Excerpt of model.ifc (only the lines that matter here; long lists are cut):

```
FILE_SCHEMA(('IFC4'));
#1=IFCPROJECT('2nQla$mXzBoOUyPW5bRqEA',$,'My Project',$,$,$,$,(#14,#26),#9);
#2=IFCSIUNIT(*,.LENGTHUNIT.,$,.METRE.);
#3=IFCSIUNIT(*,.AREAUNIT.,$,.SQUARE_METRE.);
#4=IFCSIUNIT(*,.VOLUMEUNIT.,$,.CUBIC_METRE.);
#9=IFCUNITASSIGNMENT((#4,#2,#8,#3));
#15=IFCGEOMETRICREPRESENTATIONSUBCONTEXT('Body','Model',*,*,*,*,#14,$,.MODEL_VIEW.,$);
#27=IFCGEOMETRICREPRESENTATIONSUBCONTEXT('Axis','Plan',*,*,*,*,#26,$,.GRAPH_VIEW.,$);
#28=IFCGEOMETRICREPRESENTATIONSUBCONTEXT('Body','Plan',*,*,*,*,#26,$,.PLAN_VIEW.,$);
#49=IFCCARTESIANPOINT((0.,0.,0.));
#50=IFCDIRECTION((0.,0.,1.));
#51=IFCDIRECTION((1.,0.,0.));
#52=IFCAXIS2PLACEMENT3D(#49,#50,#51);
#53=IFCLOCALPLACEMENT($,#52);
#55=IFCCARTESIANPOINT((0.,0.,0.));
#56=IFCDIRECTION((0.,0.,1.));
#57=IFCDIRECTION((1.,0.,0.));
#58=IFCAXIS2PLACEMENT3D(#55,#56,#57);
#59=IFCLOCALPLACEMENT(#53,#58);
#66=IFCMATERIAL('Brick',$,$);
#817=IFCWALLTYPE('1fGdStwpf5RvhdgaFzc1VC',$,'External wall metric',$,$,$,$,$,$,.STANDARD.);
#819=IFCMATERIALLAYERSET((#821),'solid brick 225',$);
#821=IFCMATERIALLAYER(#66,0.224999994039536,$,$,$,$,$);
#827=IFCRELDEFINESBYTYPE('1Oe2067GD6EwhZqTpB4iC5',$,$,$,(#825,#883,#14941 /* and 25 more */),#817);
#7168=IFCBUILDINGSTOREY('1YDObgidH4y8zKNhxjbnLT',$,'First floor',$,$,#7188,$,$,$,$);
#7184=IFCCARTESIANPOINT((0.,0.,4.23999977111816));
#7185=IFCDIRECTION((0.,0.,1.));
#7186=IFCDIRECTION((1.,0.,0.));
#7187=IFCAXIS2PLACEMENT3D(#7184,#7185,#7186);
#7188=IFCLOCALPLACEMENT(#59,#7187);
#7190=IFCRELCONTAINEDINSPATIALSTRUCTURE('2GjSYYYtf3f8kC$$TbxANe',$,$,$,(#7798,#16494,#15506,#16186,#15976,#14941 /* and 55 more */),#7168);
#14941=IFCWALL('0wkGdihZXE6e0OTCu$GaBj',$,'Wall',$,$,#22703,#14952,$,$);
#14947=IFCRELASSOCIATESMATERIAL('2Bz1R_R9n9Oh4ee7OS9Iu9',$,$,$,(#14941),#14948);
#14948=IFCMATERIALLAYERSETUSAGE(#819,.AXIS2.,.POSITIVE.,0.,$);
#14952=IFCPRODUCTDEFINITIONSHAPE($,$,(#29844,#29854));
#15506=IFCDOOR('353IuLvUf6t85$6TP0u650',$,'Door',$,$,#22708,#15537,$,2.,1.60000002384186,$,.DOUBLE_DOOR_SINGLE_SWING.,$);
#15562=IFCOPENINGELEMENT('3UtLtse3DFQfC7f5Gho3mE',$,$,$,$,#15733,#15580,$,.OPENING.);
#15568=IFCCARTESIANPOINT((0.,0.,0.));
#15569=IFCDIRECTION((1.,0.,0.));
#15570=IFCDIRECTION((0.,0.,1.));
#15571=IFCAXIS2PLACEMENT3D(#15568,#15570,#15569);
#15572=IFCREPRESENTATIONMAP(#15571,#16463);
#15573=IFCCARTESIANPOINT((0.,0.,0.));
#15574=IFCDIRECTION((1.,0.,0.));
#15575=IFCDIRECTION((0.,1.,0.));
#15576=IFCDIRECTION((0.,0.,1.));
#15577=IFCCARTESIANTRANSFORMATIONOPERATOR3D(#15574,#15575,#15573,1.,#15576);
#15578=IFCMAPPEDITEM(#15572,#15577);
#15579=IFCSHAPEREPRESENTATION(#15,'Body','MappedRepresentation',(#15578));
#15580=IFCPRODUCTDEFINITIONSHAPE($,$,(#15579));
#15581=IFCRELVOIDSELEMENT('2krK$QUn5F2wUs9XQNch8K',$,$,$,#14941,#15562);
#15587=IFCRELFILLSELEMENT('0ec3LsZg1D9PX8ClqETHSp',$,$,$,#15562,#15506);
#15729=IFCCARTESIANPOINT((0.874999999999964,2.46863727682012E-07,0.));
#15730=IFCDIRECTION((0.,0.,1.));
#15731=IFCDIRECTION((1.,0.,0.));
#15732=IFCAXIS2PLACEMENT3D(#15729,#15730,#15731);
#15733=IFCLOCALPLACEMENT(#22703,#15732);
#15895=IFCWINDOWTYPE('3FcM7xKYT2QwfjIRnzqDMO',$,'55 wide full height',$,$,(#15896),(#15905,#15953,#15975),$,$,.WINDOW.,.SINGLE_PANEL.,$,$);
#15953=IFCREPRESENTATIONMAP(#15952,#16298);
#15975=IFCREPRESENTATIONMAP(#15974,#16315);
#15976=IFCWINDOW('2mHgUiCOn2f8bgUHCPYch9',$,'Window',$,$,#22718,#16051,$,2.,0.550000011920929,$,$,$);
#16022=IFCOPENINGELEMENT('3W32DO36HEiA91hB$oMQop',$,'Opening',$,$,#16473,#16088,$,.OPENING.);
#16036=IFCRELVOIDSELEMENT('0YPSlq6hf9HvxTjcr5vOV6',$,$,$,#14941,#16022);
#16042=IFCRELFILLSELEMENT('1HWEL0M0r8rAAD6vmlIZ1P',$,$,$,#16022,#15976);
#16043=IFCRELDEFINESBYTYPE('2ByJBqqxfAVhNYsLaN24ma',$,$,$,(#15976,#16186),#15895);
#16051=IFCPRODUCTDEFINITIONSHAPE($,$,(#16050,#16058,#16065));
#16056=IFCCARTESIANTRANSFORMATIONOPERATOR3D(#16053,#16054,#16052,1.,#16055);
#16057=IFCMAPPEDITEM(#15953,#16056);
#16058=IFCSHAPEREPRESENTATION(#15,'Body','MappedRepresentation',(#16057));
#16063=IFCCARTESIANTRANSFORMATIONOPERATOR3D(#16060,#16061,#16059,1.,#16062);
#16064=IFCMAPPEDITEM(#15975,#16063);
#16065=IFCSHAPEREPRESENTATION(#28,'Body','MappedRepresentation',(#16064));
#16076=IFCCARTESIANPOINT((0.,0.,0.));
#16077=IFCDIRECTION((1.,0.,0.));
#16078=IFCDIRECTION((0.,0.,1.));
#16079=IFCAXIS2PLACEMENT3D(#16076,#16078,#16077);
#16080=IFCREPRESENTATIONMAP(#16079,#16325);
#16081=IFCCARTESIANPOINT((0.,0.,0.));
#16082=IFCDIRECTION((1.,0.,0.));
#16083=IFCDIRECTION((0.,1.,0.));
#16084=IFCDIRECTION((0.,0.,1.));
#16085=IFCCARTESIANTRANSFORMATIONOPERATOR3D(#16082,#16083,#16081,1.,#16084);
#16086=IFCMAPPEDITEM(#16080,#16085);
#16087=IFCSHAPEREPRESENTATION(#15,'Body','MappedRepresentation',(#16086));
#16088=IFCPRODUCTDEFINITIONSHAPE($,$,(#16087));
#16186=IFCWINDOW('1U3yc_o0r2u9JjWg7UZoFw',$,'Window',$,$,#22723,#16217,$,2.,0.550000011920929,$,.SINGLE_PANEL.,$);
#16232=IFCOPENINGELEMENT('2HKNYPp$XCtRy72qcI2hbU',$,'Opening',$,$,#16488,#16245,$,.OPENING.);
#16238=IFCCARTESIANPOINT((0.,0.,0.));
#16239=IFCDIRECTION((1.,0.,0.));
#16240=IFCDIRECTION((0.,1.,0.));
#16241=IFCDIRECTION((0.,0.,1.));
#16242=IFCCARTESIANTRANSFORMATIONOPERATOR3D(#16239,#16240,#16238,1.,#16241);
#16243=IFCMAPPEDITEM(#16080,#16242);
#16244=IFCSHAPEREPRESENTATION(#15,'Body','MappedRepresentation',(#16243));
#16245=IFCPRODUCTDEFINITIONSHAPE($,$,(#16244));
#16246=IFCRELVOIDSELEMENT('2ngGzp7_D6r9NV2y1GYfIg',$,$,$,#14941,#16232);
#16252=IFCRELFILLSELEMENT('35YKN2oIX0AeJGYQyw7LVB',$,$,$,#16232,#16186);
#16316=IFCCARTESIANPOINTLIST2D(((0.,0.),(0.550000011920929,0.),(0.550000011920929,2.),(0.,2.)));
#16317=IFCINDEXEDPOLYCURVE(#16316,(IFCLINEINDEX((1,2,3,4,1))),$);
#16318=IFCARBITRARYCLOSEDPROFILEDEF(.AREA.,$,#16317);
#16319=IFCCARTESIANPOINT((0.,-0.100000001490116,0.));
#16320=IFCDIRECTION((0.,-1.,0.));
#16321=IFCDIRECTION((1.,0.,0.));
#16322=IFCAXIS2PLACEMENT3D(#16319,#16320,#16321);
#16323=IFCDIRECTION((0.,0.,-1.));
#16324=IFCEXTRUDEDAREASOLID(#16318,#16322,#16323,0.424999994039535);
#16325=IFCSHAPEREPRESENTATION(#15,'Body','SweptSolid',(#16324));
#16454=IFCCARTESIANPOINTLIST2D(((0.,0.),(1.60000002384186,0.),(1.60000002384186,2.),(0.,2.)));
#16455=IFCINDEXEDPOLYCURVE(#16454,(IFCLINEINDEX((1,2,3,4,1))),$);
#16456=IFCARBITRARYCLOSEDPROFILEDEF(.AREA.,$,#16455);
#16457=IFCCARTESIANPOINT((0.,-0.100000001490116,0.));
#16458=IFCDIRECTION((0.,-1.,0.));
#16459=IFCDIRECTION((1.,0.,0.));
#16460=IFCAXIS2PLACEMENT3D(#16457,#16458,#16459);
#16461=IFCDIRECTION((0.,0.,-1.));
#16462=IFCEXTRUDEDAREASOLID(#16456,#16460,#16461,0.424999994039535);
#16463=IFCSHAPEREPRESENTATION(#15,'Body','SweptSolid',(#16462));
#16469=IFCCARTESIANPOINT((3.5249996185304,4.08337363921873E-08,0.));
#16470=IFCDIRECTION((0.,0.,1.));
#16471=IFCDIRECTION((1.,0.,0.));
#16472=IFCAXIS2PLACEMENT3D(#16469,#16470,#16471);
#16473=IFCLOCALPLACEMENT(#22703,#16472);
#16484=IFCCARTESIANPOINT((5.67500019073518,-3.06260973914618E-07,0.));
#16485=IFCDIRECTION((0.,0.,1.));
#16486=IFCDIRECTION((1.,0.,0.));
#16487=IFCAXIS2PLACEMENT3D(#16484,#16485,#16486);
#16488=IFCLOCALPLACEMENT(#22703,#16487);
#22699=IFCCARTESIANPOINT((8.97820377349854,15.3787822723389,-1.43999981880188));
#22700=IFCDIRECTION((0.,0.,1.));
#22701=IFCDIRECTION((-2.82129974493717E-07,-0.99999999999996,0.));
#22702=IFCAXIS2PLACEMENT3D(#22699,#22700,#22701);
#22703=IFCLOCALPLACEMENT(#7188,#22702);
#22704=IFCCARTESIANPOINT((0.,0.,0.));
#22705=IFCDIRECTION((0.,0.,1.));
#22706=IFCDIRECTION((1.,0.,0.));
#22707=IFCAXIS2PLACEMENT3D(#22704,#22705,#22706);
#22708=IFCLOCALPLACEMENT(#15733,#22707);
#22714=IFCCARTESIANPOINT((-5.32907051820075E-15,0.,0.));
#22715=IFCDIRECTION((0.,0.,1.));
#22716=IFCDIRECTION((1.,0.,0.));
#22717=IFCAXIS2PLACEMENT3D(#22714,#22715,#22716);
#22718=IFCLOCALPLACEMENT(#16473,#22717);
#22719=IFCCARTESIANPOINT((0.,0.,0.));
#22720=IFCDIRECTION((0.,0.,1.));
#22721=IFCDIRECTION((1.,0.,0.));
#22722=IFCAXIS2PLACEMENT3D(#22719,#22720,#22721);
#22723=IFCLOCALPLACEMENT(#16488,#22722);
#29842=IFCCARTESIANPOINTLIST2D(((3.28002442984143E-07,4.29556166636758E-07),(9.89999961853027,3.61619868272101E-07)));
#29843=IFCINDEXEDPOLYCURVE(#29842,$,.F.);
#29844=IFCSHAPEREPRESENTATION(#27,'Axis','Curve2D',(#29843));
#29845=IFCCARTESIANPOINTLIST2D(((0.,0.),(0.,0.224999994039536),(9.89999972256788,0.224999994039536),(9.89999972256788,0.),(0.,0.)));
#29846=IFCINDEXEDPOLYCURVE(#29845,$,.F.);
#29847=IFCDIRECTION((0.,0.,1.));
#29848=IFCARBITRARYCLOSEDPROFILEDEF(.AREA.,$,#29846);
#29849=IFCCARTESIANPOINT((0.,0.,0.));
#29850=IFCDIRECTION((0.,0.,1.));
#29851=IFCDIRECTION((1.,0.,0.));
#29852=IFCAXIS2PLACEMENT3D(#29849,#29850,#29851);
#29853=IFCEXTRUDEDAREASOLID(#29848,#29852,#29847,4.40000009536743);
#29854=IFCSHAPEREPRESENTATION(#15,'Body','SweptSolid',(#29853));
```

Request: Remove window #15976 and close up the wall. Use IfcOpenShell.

```python
import ifcopenshell
import ifcopenshell.api.feature
import ifcopenshell.api.root
import ifcopenshell.geom
import ifcopenshell.util.shape

model = ifcopenshell.open("model.ifc")
settings = ifcopenshell.geom.settings()


def volume(element):
    """Net volume in cubic metres, openings subtracted."""
    shape = ifcopenshell.geom.create_shape(settings, element)
    return ifcopenshell.util.shape.get_volume(shape.geometry)


window = model.by_guid("2mHgUiCOn2f8bgUHCPYch9")
opening = window.FillsVoids[0].RelatingOpeningElement
wall = opening.VoidsElements[0].RelatingBuildingElement
before = volume(wall)

ifcopenshell.api.root.remove_product(model, product=window)
ifcopenshell.api.feature.remove_feature(model, feature=opening)

after = volume(wall)

print(f"wall volume {before:.3f} -> {after:.3f} m3")

model.write("model_updated.ifc")
```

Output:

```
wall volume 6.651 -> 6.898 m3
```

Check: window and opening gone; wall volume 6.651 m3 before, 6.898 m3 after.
